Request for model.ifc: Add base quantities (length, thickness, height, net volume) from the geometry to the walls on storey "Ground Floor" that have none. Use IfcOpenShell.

First a look at what the model holds.

```python
import ifcopenshell
import ifcopenshell.util.element
import ifcopenshell.util.unit

model = ifcopenshell.open("model.ifc")
print(model.schema)
for unit_type in ("LENGTHUNIT", "AREAUNIT", "VOLUMEUNIT"):
    print(unit_type, ifcopenshell.util.unit.calculate_unit_scale(model, unit_type))
storey = next(s for s in model.by_type("IfcBuildingStorey") if s.Name == "Ground Floor")
walls = [e for e in ifcopenshell.util.element.get_decomposition(storey) if e.is_a("IfcWall")]
for e in sorted(walls, key=lambda e: e.id()):
    print(e.id(), e.is_a(), e.Name, list(ifcopenshell.util.element.get_psets(e, qtos_only=True)), sep=" | ")
```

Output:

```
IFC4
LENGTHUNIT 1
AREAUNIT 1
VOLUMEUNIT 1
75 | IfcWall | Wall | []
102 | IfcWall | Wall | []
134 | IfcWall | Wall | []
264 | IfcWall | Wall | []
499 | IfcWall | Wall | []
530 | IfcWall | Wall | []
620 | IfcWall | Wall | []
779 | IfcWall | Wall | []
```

```python
import ifcopenshell
import ifcopenshell.api.pset
import ifcopenshell.geom
import ifcopenshell.util.element
import ifcopenshell.util.shape
import ifcopenshell.util.unit

model = ifcopenshell.open("model.ifc")
unit_scale = ifcopenshell.util.unit.calculate_unit_scale(model)
volume_scale = ifcopenshell.util.unit.calculate_unit_scale(model, "VOLUMEUNIT")
settings = ifcopenshell.geom.settings()

storey = next(s for s in model.by_type("IfcBuildingStorey") if s.Name == "Ground Floor")
walls = [e for e in ifcopenshell.util.element.get_decomposition(storey) if e.is_a("IfcWall")]

for e in sorted(walls, key=lambda e: e.id()):
    if ifcopenshell.util.element.get_psets(e, qtos_only=True, should_inherit=False):
        continue
    # Geometry comes back in metres, in the element's own axes.
    shape = ifcopenshell.geom.create_shape(settings, e)
    values = {
        "Length": ifcopenshell.util.shape.get_x(shape.geometry) / unit_scale,
        "Width": ifcopenshell.util.shape.get_y(shape.geometry) / unit_scale,
        "Height": ifcopenshell.util.shape.get_z(shape.geometry) / unit_scale,
        "NetVolume": ifcopenshell.util.shape.get_volume(shape.geometry) / volume_scale,
    }
    qto = ifcopenshell.api.pset.add_qto(model, product=e, name="Qto_WallBaseQuantities")
    ifcopenshell.api.pset.edit_qto(model, qto=qto, properties=values)
    print(e.id(), {k: round(v, 3) for k, v in values.items()})

model.write("model_updated.ifc")
```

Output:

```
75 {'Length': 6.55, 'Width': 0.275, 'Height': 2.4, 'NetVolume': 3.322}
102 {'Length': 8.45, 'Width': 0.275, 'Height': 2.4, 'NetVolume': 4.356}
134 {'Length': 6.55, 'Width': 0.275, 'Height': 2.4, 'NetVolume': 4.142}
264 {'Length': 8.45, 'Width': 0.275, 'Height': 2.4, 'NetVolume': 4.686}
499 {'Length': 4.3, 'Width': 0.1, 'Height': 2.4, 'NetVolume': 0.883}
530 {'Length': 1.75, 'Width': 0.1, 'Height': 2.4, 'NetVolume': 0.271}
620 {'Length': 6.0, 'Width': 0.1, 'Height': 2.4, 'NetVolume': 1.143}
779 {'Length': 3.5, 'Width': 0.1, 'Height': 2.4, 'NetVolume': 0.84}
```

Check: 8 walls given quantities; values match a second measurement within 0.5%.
